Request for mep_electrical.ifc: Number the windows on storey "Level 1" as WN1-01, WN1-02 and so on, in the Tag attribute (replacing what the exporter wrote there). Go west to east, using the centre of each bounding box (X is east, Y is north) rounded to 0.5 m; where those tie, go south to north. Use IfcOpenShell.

First a look at what the model holds.

```python
import ifcopenshell
import ifcopenshell.util.element
import ifcopenshell.util.placement

model = ifcopenshell.open("mep_electrical.ifc")
print(model.schema)
storey = next(s for s in model.by_type("IfcBuildingStorey") if s.Name == "Level 1")
windows = [e for e in ifcopenshell.util.element.get_decomposition(storey) if e.is_a("IfcWindow")]
for e in sorted(windows, key=lambda e: e.id()):
    origin = ifcopenshell.util.placement.get_local_placement(e.ObjectPlacement)[:3, 3]
    print(e.id(), e.Tag, e.Name, origin.round(2) + 0.0, sep=" | ")
```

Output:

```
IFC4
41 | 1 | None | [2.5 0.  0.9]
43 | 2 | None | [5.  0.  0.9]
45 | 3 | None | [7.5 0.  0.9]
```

```python
import ifcopenshell
import ifcopenshell.geom
import ifcopenshell.util.element
import ifcopenshell.util.shape

model = ifcopenshell.open("mep_electrical.ifc")
settings = ifcopenshell.geom.settings()
settings.set("use-world-coords", True)


def centre(element):
    shape = ifcopenshell.geom.create_shape(settings, element)
    return ifcopenshell.util.shape.get_bbox_centroid(shape.geometry)


storey = next(s for s in model.by_type("IfcBuildingStorey") if s.Name == "Level 1")
windows = [e for e in ifcopenshell.util.element.get_decomposition(storey) if e.is_a("IfcWindow")]

# Insertion points can sit at a corner or the storey origin, so sort by the geometry (in metres).
centres = {e: centre(e) for e in windows}
windows.sort(key=lambda e: (round(centres[e][0] / 0.5), centres[e][1]))

for i, e in enumerate(windows, start=1):
    number = f"WN1-{i:02d}"
    e.Tag = number
    print(e.id(), number)

model.write("mep_electrical_rev.ifc")
```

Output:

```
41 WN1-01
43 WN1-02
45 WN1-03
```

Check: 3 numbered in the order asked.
